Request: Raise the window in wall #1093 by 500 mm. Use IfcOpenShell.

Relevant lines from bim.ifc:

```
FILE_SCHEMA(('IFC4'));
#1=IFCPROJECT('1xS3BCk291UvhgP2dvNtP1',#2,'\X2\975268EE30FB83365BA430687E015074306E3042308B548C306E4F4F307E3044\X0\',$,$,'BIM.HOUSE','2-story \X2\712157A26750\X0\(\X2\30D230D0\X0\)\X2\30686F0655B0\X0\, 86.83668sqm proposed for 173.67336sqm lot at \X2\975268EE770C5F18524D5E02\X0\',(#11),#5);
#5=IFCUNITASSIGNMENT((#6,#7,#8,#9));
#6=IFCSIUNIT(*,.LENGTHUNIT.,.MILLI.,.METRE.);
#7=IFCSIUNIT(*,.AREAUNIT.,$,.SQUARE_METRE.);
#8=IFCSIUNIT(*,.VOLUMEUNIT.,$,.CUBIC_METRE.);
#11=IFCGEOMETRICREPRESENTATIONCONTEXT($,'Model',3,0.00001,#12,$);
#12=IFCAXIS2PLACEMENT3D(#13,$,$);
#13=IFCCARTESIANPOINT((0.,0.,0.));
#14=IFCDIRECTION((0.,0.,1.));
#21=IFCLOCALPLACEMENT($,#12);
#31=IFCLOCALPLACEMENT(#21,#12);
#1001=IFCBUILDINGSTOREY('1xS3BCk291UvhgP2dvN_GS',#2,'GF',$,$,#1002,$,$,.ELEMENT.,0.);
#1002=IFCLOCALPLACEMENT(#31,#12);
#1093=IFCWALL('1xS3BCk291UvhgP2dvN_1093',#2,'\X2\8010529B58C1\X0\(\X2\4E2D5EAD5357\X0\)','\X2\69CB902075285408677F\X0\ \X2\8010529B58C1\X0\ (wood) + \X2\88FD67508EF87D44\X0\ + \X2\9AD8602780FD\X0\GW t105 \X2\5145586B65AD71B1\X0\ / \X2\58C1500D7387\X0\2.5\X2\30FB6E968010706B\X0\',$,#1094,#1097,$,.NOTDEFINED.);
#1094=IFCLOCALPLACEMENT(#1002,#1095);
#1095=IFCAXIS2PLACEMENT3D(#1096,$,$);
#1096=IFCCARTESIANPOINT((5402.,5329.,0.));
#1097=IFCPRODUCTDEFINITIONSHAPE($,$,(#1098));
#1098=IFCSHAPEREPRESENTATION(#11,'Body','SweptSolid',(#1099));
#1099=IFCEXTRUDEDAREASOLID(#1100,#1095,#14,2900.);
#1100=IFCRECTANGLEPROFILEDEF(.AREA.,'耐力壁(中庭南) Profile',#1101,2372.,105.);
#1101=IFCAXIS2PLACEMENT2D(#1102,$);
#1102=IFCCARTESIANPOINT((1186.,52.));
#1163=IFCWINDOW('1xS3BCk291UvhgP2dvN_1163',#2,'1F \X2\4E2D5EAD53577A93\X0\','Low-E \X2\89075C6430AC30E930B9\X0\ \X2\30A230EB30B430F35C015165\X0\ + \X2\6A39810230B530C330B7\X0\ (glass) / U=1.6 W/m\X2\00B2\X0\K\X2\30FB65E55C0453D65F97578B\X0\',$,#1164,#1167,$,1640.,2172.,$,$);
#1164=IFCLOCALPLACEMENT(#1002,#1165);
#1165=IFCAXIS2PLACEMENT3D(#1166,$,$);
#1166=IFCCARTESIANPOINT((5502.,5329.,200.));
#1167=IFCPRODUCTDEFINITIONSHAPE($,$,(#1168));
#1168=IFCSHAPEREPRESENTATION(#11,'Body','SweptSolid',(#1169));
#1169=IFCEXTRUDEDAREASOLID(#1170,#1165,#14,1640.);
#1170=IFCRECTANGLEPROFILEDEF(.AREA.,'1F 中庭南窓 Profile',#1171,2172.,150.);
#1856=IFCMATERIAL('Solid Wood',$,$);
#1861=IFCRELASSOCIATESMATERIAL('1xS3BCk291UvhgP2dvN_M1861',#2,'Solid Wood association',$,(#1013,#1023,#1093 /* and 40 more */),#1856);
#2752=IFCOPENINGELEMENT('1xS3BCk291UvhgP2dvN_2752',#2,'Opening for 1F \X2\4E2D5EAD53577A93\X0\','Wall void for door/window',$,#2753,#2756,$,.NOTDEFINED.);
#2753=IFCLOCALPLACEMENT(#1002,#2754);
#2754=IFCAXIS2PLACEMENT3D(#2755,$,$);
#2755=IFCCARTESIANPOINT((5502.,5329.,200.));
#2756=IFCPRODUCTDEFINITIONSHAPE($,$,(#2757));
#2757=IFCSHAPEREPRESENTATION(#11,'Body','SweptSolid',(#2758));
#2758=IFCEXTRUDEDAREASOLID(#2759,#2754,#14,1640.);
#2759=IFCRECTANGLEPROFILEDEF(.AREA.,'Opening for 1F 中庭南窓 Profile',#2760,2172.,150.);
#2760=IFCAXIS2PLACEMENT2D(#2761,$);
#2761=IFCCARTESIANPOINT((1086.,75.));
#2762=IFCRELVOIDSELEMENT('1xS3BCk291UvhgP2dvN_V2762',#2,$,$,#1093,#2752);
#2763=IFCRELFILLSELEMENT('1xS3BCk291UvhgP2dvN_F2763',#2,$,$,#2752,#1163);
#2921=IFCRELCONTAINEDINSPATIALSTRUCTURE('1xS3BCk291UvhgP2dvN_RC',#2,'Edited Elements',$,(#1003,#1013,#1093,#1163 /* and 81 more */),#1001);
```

```python
import numpy as np
import ifcopenshell
import ifcopenshell.api.geometry
import ifcopenshell.util.placement
import ifcopenshell.util.unit

model = ifcopenshell.open("bim.ifc")
unit_scale = ifcopenshell.util.unit.calculate_unit_scale(model)

window = model.by_guid("1xS3BCk291UvhgP2dvN_1163")
opening = window.FillsVoids[0].RelatingOpeningElement
dz = 0.5 / unit_scale

shift = np.array([0.0, 0.0, dz])
# The window is not placed relative to its opening, so move both.
for product in (opening, window):
    matrix = ifcopenshell.util.placement.get_local_placement(product.ObjectPlacement)
    matrix[:3, 3] += shift
    ifcopenshell.api.geometry.edit_object_placement(model, product=product, matrix=matrix, is_si=False)

print(f"moved by {dz * unit_scale:+.3f} m")

model.write("bim_edited.ifc")
```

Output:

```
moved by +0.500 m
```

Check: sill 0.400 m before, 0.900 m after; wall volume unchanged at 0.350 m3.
